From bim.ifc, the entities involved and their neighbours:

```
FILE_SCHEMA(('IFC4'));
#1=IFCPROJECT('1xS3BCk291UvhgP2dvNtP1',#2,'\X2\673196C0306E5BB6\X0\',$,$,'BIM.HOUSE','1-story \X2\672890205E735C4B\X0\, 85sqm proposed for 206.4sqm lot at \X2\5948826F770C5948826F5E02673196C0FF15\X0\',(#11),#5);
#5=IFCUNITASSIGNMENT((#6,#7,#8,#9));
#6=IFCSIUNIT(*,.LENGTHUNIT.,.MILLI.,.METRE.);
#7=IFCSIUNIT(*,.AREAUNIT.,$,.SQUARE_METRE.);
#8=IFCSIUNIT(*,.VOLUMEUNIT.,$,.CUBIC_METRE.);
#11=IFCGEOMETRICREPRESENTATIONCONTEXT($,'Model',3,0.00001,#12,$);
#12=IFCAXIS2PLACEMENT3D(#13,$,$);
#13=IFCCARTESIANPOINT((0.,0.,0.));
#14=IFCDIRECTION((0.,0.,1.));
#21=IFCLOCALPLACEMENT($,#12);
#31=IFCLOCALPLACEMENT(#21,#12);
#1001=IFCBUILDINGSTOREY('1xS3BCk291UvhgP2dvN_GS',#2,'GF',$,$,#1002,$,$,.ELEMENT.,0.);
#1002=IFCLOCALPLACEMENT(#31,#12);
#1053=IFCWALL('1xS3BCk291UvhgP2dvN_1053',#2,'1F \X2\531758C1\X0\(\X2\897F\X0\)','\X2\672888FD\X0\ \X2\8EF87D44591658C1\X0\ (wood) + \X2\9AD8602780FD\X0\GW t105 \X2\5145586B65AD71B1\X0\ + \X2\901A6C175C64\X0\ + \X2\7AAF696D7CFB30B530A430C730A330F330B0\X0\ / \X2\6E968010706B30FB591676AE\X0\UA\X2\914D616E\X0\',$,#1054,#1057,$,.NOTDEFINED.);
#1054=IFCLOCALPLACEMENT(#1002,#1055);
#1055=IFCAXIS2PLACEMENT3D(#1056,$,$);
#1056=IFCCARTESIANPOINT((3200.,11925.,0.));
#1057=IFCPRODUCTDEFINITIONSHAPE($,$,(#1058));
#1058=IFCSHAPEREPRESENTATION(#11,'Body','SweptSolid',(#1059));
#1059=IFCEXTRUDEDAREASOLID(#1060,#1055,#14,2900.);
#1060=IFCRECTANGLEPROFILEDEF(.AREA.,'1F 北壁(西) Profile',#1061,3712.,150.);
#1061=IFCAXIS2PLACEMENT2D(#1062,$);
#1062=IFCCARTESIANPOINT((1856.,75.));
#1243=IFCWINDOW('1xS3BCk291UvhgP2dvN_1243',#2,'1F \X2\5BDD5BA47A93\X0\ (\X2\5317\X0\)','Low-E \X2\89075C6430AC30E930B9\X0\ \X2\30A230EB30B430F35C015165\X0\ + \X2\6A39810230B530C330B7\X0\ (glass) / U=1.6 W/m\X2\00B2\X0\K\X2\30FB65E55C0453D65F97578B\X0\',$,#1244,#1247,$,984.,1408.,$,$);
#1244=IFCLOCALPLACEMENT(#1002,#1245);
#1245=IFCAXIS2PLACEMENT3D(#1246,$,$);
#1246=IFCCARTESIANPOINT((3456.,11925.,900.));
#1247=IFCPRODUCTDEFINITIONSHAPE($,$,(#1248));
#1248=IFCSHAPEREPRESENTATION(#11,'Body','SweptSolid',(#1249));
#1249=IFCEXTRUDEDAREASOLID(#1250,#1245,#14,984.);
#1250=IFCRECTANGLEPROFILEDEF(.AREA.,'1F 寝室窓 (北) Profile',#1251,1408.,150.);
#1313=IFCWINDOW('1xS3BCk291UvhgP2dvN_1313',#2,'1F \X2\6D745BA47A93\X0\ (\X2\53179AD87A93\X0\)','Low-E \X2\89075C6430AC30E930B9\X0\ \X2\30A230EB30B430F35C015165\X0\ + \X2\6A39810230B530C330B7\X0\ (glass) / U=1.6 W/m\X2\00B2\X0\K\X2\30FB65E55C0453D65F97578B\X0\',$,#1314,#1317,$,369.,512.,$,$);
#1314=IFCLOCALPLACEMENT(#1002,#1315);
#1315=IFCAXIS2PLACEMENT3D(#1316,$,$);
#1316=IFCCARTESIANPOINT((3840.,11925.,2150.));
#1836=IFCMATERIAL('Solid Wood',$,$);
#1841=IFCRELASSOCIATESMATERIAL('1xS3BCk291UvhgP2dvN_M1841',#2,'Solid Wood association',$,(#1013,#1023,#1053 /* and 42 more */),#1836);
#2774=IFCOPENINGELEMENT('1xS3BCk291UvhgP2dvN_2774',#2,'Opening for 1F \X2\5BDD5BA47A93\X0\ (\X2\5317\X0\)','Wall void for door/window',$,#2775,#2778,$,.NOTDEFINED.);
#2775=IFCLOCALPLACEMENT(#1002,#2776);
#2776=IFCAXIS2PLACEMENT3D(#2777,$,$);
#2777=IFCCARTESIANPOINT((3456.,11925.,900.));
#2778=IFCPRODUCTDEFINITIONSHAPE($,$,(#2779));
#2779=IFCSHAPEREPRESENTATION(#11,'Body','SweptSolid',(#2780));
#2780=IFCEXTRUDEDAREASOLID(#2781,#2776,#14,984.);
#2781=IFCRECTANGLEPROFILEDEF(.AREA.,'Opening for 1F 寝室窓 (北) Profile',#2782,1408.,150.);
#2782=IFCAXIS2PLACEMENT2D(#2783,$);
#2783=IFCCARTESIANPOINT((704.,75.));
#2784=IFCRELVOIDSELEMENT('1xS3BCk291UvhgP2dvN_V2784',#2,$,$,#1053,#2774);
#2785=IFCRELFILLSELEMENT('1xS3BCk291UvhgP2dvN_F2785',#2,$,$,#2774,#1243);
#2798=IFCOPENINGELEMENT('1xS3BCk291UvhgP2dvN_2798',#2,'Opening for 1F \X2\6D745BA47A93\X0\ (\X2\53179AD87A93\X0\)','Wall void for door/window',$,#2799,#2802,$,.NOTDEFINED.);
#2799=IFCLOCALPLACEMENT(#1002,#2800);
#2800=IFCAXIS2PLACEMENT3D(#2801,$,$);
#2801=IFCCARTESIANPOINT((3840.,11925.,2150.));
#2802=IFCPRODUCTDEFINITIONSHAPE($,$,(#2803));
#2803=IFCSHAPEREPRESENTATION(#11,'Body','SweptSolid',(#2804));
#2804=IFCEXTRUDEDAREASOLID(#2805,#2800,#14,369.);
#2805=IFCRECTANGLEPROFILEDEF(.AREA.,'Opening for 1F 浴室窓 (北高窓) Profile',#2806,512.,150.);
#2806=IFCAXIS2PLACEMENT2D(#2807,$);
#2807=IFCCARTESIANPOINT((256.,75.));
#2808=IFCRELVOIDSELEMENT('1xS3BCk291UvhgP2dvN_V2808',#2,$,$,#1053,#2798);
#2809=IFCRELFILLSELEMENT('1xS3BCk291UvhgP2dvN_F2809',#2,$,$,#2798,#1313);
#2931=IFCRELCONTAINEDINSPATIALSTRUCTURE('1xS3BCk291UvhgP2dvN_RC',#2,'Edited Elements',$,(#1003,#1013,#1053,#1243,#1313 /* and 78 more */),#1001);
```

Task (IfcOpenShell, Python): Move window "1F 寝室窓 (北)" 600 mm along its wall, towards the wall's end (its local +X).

```python
import ifcopenshell
import ifcopenshell.api.geometry
import ifcopenshell.util.placement
import ifcopenshell.util.unit

model = ifcopenshell.open("bim.ifc")
unit_scale = ifcopenshell.util.unit.calculate_unit_scale(model)

window = model.by_guid("1xS3BCk291UvhgP2dvN_1243")
opening = window.FillsVoids[0].RelatingOpeningElement
wall = opening.VoidsElements[0].RelatingBuildingElement

wall_matrix = ifcopenshell.util.placement.get_local_placement(wall.ObjectPlacement)
shift = wall_matrix[:3, 0] * 0.6 / unit_scale
before = ifcopenshell.util.placement.get_local_placement(window.ObjectPlacement)[:3, 3].copy()

# The window is not placed relative to its opening, so move both.
for product in (opening, window):
    matrix = ifcopenshell.util.placement.get_local_placement(product.ObjectPlacement)
    matrix[:3, 3] += shift
    ifcopenshell.api.geometry.edit_object_placement(model, product=product, matrix=matrix, is_si=False)

after = ifcopenshell.util.placement.get_local_placement(window.ObjectPlacement)[:3, 3]
print("window moved by", (after - before).round(3) + 0.0)

model.write("bim_v2.ifc")
```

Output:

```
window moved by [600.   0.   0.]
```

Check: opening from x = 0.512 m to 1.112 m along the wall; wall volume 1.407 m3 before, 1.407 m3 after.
